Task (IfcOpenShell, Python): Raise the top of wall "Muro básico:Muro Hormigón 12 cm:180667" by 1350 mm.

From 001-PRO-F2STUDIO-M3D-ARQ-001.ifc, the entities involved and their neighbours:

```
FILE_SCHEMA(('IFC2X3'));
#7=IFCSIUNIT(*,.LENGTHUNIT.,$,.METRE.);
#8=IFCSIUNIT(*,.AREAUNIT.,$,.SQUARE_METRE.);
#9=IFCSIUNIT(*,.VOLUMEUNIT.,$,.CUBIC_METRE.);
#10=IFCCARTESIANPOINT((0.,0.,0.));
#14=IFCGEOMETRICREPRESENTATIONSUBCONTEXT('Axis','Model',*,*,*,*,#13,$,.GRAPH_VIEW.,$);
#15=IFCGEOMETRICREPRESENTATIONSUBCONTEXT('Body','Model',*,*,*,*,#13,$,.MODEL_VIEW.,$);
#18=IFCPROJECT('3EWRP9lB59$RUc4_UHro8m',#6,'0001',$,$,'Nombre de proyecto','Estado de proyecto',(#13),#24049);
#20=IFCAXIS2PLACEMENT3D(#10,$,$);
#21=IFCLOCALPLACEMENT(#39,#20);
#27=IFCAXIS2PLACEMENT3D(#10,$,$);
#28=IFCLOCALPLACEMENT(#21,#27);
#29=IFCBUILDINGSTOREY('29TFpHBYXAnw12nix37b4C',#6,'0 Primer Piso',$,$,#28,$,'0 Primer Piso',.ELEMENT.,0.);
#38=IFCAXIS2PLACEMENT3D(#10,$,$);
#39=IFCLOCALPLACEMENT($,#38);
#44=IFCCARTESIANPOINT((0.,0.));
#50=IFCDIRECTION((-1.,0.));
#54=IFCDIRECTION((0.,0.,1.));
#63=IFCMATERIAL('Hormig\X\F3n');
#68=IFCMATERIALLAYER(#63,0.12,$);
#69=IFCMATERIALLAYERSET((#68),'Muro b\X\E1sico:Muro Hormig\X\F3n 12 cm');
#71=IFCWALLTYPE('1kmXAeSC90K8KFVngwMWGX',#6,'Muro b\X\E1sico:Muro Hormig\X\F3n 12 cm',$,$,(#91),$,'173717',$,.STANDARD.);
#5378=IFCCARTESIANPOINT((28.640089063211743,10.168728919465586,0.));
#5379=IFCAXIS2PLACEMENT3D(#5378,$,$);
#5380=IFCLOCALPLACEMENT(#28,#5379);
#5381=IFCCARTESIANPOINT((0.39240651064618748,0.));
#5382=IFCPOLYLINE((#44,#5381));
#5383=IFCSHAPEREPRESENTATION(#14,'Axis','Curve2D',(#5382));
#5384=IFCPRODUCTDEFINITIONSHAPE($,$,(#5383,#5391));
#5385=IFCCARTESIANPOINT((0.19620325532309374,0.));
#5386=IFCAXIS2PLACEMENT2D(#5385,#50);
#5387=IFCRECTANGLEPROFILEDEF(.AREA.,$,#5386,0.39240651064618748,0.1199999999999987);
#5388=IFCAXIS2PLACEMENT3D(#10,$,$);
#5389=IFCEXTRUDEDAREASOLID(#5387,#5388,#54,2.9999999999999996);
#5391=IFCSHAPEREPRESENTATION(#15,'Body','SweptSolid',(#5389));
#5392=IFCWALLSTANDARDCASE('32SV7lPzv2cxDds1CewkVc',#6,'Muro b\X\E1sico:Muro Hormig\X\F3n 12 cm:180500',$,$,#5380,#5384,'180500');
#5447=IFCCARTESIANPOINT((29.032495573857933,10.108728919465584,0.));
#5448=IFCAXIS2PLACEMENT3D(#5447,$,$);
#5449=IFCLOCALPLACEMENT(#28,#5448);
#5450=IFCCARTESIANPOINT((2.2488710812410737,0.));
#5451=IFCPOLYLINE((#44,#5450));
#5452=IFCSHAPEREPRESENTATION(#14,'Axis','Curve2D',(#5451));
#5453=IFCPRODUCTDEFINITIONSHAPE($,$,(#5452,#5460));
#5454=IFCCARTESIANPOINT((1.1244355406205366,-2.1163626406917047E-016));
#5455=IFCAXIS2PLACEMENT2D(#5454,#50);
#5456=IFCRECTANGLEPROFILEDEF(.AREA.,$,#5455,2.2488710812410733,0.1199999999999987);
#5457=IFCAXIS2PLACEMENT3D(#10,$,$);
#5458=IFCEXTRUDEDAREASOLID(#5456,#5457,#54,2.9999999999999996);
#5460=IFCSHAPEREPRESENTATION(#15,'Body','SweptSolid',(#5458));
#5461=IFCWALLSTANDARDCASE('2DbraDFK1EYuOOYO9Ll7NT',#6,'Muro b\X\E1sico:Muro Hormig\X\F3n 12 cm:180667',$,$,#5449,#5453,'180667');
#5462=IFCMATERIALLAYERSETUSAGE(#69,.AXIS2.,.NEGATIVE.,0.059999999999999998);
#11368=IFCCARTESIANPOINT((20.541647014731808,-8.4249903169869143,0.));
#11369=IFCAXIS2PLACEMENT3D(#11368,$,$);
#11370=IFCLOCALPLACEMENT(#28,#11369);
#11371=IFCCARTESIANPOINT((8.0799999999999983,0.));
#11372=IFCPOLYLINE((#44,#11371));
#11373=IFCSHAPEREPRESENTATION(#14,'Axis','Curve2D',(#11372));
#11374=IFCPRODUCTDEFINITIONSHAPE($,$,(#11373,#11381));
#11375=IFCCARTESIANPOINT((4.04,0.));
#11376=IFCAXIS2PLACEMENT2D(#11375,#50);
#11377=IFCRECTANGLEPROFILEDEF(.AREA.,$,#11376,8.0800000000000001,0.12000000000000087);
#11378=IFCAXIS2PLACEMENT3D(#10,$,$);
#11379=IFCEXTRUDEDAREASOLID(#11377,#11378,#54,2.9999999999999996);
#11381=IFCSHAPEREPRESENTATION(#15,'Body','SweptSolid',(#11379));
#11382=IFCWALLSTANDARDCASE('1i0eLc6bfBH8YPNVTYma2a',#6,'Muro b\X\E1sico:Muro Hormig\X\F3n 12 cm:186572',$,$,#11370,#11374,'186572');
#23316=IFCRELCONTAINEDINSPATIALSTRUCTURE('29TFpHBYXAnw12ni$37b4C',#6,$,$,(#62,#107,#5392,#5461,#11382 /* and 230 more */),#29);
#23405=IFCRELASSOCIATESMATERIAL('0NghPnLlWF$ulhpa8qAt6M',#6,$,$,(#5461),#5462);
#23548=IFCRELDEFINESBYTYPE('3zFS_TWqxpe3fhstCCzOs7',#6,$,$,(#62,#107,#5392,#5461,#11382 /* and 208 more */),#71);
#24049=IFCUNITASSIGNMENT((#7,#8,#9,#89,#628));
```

```python
import ifcopenshell
import ifcopenshell.geom
import ifcopenshell.util.representation
import ifcopenshell.util.shape
import ifcopenshell.util.unit

model = ifcopenshell.open("001-PRO-F2STUDIO-M3D-ARQ-001.ifc")
unit_scale = ifcopenshell.util.unit.calculate_unit_scale(model)
settings = ifcopenshell.geom.settings()


def volume(element):
    """Net volume in cubic metres, openings subtracted."""
    shape = ifcopenshell.geom.create_shape(settings, element)
    return ifcopenshell.util.shape.get_volume(shape.geometry)


wall = model.by_guid("2DbraDFK1EYuOOYO9Ll7NT")
before = volume(wall)

body = ifcopenshell.util.representation.get_representation(wall, "Model", "Body")
solid = body.Items[0]
old_height = solid.Depth
solid.Depth += 1.35 / unit_scale
after = volume(wall)

print(f"height {old_height:g} -> {solid.Depth:g}, volume {before:.3f} -> {after:.3f} m3")

model.write("001-PRO-F2STUDIO-M3D-ARQ-001_rev.ifc")
```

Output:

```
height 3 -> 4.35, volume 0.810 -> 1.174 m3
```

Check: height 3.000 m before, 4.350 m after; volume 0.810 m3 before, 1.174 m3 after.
